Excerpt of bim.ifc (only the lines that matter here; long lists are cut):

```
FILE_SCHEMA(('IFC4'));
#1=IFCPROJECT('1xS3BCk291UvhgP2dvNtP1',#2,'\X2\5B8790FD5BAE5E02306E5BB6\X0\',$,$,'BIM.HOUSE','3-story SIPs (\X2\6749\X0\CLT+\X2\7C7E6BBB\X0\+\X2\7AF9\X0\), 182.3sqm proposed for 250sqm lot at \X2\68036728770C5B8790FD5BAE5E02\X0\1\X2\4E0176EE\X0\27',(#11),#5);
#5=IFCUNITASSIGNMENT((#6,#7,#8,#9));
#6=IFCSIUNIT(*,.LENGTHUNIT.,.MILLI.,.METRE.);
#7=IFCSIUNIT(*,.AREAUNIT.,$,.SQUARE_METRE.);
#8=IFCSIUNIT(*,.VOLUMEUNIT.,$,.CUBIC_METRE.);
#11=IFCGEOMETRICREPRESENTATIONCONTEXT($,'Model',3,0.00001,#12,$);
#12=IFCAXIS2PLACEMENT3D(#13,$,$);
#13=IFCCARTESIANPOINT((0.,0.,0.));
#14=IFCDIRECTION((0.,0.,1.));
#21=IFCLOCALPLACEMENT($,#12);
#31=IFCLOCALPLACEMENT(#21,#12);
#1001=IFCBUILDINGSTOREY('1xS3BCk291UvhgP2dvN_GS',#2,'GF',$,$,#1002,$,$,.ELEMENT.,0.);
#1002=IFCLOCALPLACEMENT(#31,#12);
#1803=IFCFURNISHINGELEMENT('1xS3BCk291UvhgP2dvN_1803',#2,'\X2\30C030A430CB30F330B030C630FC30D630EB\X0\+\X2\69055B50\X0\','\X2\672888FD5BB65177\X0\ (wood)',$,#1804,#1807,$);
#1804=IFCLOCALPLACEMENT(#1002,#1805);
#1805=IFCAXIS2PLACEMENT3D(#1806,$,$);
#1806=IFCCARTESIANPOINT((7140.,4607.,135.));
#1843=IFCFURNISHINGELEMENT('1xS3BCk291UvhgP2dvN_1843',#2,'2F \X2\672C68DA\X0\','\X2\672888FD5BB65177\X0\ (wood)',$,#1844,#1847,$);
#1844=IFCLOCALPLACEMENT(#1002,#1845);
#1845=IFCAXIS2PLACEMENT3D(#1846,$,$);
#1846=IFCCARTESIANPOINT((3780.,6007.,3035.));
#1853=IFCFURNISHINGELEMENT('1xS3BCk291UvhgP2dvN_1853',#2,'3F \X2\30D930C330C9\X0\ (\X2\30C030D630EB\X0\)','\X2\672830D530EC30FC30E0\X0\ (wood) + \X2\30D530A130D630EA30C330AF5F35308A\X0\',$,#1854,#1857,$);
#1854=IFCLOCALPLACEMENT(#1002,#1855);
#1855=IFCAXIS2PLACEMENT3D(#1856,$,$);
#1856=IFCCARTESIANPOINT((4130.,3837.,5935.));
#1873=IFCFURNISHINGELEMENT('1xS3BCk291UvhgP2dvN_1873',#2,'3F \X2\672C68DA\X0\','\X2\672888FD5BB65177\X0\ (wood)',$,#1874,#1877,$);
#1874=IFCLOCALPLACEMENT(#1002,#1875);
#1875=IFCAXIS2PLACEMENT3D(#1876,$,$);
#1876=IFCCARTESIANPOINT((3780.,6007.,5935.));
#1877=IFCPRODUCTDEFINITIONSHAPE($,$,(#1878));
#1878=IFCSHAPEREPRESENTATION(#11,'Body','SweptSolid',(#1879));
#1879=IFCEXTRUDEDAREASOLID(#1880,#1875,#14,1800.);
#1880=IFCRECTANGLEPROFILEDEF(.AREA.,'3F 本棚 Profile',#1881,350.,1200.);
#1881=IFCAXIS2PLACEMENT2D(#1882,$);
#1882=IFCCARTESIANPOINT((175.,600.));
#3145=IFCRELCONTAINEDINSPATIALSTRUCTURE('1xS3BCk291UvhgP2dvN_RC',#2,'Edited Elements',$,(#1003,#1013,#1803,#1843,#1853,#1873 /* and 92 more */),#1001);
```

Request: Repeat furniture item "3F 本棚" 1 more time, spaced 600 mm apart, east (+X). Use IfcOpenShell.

```python
import numpy as np
import ifcopenshell
import ifcopenshell.api.geometry
import ifcopenshell.api.root
import ifcopenshell.util.element
import ifcopenshell.util.placement
import ifcopenshell.util.unit

model = ifcopenshell.open("bim.ifc")
unit_scale = ifcopenshell.util.unit.calculate_unit_scale(model)


def reuse_history(source, copy):
    """copy_class also copies each property set's owner history, people and application; keep the originals."""
    for rel in copy.IsDefinedBy:
        if rel.is_a("IfcRelDefinesByProperties") and (history := rel.RelatingPropertyDefinition.OwnerHistory):
            rel.RelatingPropertyDefinition.OwnerHistory = source.OwnerHistory
            ifcopenshell.util.element.remove_deep2(model, history)


source = model.by_id(1873)
base = ifcopenshell.util.placement.get_local_placement(source.ObjectPlacement)
step = np.array([1.0, 0.0, 0.0]) * 0.6 / unit_scale

for i in range(1, 2):
    copy = ifcopenshell.api.root.copy_class(model, product=source)
    copy.Representation = ifcopenshell.util.element.copy_deep(
        model, source.Representation, exclude=["IfcGeometricRepresentationContext", "IfcRepresentationMap"]
    )
    reuse_history(source, copy)
    matrix = base.copy()
    matrix[:3, 3] += i * step
    print("added at", matrix[:3, 3].round(3) + 0.0)
    ifcopenshell.api.geometry.edit_object_placement(model, product=copy, matrix=matrix, is_si=False)

model.write("bim_rev.ifc")
```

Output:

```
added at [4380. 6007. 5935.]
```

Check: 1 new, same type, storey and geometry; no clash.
